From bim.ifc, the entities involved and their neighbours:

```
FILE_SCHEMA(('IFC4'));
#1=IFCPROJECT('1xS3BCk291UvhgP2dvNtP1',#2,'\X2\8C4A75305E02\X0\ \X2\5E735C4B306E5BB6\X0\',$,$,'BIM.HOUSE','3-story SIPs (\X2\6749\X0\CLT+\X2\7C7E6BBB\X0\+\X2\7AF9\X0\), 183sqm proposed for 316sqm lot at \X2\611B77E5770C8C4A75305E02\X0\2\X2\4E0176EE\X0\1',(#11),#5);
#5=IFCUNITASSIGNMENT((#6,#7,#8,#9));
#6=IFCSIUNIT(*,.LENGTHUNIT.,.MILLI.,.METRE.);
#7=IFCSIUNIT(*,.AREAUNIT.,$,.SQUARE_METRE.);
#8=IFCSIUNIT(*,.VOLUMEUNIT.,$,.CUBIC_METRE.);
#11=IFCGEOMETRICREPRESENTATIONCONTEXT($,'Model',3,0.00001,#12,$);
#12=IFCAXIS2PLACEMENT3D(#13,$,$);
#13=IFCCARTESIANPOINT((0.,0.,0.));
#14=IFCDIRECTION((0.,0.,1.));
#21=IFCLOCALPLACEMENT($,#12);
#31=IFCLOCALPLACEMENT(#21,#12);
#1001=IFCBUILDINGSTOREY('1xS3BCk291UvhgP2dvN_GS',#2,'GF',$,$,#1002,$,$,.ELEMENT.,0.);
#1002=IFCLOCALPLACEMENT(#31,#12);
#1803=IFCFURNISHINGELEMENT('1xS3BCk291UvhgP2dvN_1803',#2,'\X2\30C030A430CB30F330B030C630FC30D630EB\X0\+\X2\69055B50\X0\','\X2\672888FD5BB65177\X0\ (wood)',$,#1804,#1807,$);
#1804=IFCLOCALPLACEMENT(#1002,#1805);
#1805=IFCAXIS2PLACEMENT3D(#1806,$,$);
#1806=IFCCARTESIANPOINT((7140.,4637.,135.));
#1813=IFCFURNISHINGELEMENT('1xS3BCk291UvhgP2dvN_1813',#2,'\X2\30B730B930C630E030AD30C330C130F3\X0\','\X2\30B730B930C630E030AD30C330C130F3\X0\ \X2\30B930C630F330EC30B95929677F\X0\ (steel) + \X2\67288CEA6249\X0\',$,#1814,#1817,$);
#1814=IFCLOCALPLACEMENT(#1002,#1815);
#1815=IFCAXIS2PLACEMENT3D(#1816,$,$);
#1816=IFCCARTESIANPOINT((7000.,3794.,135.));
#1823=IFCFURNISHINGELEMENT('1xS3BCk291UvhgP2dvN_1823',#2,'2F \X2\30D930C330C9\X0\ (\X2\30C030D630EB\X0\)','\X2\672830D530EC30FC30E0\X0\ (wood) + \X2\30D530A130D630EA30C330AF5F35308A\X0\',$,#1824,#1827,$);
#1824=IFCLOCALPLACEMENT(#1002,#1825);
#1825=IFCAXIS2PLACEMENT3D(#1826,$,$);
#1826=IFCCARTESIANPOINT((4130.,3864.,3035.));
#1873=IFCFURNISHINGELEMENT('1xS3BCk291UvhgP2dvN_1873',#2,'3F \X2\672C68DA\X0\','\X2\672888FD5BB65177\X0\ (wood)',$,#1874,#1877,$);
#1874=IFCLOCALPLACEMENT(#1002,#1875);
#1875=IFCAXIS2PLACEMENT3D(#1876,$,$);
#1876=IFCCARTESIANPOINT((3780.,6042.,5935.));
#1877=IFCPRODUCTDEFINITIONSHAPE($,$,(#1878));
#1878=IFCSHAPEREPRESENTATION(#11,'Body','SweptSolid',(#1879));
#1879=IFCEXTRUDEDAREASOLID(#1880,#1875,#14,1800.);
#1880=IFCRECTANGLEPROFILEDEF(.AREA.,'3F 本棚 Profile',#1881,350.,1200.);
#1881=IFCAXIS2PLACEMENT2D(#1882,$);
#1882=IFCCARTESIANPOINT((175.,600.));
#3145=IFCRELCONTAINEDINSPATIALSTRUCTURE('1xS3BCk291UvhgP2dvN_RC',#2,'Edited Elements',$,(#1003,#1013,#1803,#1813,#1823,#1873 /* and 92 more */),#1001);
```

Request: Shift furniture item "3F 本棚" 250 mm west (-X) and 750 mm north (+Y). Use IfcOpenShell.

```python
import ifcopenshell
import ifcopenshell.api.geometry
import ifcopenshell.util.placement

model = ifcopenshell.open("bim.ifc")

item = model.by_guid("1xS3BCk291UvhgP2dvN_1873")
matrix = ifcopenshell.util.placement.get_local_placement(item.ObjectPlacement)
matrix[0, 3] -= 250.0
matrix[1, 3] += 750.0
ifcopenshell.api.geometry.edit_object_placement(model, product=item, matrix=matrix, is_si=False)

print(ifcopenshell.util.placement.get_local_placement(item.ObjectPlacement).round(3) + 0.0)

model.write("bim_updated.ifc")
```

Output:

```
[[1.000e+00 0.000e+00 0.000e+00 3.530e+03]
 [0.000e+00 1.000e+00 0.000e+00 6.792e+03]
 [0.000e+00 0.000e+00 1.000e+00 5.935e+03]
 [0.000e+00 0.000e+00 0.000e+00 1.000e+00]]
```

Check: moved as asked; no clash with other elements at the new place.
